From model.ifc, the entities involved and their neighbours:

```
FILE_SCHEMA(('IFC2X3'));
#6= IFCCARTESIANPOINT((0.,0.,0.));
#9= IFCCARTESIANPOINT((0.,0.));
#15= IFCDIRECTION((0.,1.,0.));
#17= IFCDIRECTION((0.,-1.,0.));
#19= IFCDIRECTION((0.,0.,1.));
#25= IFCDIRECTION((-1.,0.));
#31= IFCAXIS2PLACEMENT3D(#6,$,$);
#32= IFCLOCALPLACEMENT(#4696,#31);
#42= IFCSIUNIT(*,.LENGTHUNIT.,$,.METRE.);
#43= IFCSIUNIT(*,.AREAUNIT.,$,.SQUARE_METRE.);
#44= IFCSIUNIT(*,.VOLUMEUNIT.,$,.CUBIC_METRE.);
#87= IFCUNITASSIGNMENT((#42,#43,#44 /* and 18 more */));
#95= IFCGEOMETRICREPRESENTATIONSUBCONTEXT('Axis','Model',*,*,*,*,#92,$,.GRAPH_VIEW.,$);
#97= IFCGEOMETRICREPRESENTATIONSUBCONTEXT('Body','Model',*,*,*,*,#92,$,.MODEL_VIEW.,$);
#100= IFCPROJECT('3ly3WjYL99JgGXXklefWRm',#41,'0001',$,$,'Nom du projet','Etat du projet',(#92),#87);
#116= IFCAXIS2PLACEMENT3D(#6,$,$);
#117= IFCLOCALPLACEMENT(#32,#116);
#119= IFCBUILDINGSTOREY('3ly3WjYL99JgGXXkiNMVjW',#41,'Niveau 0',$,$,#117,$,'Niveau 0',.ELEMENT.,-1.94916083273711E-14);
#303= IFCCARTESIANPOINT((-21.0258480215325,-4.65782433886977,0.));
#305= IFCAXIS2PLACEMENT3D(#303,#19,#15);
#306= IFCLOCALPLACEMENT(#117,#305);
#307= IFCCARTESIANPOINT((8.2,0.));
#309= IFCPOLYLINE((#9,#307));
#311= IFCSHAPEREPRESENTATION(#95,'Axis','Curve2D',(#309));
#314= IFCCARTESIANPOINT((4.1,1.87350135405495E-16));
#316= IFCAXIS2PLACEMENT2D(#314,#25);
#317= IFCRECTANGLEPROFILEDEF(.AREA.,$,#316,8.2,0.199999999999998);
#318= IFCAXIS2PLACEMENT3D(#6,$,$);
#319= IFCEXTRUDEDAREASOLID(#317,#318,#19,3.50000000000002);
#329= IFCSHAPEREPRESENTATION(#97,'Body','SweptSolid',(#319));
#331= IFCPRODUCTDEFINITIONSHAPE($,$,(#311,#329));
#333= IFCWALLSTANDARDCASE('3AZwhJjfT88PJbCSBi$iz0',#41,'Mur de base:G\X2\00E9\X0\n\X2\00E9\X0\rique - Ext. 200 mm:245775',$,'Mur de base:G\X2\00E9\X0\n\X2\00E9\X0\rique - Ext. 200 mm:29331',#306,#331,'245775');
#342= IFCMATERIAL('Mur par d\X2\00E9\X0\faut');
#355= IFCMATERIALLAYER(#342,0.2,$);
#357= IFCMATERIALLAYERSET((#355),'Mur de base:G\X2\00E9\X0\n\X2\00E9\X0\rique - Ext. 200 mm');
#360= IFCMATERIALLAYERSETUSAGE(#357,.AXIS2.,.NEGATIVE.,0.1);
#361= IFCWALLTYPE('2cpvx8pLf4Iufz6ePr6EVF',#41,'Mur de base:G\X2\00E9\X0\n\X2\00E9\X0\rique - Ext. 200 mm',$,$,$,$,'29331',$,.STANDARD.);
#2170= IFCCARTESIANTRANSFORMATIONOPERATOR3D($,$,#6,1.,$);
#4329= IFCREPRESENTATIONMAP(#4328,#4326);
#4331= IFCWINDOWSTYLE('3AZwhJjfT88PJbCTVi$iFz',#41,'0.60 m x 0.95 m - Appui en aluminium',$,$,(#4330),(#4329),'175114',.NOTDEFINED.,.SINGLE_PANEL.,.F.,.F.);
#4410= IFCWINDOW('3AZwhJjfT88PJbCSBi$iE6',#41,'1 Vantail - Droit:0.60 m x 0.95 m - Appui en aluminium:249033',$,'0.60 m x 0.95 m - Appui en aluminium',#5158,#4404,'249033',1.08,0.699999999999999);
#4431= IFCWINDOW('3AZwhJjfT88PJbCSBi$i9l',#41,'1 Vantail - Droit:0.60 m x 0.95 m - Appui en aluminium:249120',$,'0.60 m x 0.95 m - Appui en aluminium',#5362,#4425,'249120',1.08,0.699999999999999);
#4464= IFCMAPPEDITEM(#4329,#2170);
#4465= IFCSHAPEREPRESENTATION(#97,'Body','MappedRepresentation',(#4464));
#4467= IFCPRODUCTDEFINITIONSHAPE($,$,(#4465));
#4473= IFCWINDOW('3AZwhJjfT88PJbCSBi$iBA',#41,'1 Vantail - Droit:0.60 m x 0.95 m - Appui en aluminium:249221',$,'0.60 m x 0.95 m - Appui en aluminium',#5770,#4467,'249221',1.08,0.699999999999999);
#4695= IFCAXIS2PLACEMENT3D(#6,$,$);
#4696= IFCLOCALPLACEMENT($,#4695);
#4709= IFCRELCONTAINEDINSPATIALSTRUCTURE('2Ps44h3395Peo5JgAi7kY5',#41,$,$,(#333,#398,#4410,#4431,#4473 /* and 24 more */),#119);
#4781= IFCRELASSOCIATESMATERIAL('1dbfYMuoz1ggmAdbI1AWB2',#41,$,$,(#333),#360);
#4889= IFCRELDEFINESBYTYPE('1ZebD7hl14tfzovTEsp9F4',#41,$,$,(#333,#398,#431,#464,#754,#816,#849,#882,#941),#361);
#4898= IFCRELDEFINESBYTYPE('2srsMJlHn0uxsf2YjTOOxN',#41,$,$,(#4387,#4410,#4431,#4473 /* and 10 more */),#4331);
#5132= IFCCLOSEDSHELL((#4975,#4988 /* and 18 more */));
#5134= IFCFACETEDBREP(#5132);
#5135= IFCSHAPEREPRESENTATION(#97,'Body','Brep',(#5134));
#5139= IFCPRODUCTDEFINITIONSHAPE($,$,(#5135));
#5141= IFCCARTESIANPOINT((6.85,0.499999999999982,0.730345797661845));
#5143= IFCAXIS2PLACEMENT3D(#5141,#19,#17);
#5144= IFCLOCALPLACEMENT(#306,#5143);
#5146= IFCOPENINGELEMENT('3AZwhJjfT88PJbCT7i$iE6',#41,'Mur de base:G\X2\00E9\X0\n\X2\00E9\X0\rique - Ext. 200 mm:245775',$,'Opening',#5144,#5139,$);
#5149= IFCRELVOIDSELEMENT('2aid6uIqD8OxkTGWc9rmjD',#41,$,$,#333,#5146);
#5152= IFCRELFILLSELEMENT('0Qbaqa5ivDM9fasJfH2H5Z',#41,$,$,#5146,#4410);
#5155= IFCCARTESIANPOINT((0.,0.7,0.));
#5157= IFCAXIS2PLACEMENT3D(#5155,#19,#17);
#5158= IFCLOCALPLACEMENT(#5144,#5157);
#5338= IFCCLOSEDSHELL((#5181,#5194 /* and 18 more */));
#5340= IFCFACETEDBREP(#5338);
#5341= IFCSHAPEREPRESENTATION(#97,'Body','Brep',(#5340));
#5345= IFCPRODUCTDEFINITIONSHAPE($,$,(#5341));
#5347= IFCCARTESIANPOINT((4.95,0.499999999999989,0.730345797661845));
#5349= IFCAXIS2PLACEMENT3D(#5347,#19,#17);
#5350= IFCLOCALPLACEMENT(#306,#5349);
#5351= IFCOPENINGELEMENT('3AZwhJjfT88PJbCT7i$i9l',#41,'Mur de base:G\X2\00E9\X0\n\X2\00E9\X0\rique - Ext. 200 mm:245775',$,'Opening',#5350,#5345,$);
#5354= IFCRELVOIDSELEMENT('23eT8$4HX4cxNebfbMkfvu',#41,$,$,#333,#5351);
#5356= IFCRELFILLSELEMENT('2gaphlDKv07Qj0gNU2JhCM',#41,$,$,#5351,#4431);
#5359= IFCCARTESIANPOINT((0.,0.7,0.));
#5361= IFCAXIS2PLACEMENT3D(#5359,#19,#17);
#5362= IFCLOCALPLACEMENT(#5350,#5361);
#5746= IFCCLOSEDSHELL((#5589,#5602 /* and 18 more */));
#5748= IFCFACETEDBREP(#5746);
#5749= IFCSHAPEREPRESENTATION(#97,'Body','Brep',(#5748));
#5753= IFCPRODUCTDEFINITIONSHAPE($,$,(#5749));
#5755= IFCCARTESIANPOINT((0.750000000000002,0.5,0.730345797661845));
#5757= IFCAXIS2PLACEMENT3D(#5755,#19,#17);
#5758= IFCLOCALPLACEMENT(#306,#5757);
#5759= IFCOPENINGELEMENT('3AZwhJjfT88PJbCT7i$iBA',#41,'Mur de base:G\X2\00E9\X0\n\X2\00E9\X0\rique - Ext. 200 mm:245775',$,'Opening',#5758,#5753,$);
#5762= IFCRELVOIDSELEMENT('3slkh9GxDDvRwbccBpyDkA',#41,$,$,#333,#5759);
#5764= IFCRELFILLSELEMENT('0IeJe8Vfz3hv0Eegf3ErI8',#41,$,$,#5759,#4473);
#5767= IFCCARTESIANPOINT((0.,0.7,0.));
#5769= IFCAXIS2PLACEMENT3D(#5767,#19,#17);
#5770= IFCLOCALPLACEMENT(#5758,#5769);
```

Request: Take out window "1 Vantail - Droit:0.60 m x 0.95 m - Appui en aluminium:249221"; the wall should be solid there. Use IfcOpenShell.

```python
import ifcopenshell
import ifcopenshell.api.feature
import ifcopenshell.api.root
import ifcopenshell.geom
import ifcopenshell.util.shape

model = ifcopenshell.open("model.ifc")
settings = ifcopenshell.geom.settings()


def volume(element):
    """Net volume in cubic metres, openings subtracted."""
    shape = ifcopenshell.geom.create_shape(settings, element)
    return ifcopenshell.util.shape.get_volume(shape.geometry)


window = model.by_id(4473)
opening = window.FillsVoids[0].RelatingOpeningElement
wall = opening.VoidsElements[0].RelatingBuildingElement
before = volume(wall)

ifcopenshell.api.root.remove_product(model, product=window)
ifcopenshell.api.feature.remove_feature(model, feature=opening)

after = volume(wall)

print(f"wall volume {before:.3f} -> {after:.3f} m3")

model.write("model_edited.ifc")
```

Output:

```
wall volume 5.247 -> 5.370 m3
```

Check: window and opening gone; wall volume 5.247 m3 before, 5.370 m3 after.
